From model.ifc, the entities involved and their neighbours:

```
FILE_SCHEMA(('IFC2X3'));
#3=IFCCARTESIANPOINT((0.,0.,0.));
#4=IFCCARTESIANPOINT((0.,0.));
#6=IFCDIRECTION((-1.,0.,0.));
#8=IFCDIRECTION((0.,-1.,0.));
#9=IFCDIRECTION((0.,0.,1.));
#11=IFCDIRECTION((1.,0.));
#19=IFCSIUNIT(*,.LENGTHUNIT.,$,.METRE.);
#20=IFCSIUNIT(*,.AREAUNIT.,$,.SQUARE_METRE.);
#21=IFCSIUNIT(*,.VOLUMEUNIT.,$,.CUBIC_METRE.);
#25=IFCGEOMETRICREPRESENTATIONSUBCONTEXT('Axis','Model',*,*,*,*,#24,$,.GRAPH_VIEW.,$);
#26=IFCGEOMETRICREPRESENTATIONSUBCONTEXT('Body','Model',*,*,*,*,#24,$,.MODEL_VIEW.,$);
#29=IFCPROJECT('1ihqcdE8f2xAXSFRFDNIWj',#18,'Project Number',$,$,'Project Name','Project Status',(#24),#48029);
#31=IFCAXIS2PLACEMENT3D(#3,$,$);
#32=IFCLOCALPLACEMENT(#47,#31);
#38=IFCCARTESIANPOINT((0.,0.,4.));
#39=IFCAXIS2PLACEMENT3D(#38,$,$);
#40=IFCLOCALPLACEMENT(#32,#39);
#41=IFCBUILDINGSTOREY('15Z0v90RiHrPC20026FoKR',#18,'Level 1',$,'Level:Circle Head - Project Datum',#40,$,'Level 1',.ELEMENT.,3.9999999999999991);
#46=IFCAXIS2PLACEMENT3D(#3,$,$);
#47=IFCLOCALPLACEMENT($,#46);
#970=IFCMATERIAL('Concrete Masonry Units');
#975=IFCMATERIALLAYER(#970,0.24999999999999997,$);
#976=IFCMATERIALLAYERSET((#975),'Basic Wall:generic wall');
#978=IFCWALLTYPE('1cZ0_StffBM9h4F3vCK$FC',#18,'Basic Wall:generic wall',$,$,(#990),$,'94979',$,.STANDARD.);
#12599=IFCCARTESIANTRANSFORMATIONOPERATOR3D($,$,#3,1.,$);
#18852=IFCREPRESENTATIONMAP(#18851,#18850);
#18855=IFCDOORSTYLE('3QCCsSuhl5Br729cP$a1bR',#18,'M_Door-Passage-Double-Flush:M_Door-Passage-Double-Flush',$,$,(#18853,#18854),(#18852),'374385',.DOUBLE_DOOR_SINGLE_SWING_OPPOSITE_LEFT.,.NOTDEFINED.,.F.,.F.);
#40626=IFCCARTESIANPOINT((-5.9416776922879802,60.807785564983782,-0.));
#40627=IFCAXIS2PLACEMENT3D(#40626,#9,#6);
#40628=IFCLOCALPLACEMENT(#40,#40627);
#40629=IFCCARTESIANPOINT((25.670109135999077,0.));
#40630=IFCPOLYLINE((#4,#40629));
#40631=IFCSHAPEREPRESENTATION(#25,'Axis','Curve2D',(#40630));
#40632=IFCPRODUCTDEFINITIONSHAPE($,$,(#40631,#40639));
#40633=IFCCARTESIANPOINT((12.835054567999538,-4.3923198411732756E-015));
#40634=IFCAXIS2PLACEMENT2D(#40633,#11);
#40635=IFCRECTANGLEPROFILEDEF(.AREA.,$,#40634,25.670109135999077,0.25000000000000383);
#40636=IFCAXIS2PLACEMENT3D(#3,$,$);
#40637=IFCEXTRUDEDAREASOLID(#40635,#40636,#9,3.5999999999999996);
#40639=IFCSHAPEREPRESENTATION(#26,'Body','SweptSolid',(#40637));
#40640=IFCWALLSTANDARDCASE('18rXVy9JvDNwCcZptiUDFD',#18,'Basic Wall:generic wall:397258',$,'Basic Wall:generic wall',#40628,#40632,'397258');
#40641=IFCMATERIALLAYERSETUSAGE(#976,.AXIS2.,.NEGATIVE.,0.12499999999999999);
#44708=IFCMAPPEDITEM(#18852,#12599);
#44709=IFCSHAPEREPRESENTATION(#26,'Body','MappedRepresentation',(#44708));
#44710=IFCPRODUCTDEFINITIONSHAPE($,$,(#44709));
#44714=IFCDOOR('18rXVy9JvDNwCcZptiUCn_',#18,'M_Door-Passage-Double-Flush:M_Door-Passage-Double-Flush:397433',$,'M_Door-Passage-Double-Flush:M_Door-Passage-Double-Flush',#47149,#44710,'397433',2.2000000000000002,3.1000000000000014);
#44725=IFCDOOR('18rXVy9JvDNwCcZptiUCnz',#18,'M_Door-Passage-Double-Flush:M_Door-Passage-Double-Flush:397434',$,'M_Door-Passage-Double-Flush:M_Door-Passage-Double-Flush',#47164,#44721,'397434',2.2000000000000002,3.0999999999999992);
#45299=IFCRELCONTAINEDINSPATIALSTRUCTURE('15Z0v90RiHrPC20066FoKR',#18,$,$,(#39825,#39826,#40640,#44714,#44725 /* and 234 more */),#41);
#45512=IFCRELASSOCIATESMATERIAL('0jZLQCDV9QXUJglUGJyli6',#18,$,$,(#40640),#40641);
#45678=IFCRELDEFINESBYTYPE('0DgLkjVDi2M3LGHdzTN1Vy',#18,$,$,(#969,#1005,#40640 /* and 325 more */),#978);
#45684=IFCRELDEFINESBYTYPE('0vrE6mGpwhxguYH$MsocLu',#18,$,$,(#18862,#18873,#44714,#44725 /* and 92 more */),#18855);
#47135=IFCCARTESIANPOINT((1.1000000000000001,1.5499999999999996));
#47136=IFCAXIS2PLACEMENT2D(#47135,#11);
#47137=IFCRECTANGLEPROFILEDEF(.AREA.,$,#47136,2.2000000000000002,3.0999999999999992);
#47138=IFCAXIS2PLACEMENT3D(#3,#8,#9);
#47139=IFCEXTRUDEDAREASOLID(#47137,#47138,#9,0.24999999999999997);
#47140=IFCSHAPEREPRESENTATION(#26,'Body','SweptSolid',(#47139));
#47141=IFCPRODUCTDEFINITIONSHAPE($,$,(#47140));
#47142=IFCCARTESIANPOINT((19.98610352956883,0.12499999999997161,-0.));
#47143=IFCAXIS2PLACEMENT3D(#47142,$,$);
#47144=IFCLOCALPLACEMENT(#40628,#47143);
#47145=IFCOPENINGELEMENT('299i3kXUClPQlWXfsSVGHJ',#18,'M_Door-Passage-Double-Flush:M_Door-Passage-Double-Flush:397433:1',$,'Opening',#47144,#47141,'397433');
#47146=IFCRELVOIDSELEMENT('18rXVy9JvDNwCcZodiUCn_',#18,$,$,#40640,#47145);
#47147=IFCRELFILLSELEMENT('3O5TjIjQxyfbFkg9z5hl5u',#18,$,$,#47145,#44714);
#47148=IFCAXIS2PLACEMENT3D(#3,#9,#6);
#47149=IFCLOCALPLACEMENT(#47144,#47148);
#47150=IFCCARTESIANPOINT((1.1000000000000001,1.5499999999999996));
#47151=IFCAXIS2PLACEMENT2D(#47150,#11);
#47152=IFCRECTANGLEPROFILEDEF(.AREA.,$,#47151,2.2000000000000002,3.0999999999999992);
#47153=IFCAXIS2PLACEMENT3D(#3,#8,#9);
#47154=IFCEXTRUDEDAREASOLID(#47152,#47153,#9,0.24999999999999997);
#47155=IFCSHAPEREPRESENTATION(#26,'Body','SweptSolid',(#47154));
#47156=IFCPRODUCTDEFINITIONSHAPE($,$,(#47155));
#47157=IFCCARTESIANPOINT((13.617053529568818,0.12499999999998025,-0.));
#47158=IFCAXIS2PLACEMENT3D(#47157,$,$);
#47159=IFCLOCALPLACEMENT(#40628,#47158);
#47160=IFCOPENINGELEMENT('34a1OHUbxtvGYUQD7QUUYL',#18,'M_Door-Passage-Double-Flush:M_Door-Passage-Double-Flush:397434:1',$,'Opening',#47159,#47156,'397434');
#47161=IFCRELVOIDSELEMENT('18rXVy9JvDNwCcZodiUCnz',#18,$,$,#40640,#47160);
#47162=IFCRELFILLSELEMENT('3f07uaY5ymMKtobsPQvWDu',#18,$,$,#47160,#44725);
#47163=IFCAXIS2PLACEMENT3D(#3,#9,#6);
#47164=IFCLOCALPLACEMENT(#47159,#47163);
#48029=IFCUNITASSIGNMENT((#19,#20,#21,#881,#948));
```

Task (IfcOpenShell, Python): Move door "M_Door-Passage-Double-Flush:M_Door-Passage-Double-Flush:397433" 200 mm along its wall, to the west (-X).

```python
import ifcopenshell
import ifcopenshell.api.geometry
import ifcopenshell.util.placement
import ifcopenshell.util.unit

model = ifcopenshell.open("model.ifc")
unit_scale = ifcopenshell.util.unit.calculate_unit_scale(model)

door = model.by_id(44714)
opening = door.FillsVoids[0].RelatingOpeningElement
wall = opening.VoidsElements[0].RelatingBuildingElement

wall_matrix = ifcopenshell.util.placement.get_local_placement(wall.ObjectPlacement)
shift = wall_matrix[:3, 0] * 0.2 / unit_scale
before = ifcopenshell.util.placement.get_local_placement(door.ObjectPlacement)[:3, 3].copy()

# The door is placed relative to its opening, so it follows when the opening moves.
matrix = ifcopenshell.util.placement.get_local_placement(opening.ObjectPlacement)
matrix[:3, 3] += shift
ifcopenshell.api.geometry.edit_object_placement(
    model, product=opening, matrix=matrix, is_si=False, should_transform_children=True
)

after = ifcopenshell.util.placement.get_local_placement(door.ObjectPlacement)[:3, 3]
print("door moved by", (after - before).round(3) + 0.0)

model.write("model_rev.ifc")
```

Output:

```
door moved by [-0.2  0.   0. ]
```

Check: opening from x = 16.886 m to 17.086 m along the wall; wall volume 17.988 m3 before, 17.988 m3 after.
